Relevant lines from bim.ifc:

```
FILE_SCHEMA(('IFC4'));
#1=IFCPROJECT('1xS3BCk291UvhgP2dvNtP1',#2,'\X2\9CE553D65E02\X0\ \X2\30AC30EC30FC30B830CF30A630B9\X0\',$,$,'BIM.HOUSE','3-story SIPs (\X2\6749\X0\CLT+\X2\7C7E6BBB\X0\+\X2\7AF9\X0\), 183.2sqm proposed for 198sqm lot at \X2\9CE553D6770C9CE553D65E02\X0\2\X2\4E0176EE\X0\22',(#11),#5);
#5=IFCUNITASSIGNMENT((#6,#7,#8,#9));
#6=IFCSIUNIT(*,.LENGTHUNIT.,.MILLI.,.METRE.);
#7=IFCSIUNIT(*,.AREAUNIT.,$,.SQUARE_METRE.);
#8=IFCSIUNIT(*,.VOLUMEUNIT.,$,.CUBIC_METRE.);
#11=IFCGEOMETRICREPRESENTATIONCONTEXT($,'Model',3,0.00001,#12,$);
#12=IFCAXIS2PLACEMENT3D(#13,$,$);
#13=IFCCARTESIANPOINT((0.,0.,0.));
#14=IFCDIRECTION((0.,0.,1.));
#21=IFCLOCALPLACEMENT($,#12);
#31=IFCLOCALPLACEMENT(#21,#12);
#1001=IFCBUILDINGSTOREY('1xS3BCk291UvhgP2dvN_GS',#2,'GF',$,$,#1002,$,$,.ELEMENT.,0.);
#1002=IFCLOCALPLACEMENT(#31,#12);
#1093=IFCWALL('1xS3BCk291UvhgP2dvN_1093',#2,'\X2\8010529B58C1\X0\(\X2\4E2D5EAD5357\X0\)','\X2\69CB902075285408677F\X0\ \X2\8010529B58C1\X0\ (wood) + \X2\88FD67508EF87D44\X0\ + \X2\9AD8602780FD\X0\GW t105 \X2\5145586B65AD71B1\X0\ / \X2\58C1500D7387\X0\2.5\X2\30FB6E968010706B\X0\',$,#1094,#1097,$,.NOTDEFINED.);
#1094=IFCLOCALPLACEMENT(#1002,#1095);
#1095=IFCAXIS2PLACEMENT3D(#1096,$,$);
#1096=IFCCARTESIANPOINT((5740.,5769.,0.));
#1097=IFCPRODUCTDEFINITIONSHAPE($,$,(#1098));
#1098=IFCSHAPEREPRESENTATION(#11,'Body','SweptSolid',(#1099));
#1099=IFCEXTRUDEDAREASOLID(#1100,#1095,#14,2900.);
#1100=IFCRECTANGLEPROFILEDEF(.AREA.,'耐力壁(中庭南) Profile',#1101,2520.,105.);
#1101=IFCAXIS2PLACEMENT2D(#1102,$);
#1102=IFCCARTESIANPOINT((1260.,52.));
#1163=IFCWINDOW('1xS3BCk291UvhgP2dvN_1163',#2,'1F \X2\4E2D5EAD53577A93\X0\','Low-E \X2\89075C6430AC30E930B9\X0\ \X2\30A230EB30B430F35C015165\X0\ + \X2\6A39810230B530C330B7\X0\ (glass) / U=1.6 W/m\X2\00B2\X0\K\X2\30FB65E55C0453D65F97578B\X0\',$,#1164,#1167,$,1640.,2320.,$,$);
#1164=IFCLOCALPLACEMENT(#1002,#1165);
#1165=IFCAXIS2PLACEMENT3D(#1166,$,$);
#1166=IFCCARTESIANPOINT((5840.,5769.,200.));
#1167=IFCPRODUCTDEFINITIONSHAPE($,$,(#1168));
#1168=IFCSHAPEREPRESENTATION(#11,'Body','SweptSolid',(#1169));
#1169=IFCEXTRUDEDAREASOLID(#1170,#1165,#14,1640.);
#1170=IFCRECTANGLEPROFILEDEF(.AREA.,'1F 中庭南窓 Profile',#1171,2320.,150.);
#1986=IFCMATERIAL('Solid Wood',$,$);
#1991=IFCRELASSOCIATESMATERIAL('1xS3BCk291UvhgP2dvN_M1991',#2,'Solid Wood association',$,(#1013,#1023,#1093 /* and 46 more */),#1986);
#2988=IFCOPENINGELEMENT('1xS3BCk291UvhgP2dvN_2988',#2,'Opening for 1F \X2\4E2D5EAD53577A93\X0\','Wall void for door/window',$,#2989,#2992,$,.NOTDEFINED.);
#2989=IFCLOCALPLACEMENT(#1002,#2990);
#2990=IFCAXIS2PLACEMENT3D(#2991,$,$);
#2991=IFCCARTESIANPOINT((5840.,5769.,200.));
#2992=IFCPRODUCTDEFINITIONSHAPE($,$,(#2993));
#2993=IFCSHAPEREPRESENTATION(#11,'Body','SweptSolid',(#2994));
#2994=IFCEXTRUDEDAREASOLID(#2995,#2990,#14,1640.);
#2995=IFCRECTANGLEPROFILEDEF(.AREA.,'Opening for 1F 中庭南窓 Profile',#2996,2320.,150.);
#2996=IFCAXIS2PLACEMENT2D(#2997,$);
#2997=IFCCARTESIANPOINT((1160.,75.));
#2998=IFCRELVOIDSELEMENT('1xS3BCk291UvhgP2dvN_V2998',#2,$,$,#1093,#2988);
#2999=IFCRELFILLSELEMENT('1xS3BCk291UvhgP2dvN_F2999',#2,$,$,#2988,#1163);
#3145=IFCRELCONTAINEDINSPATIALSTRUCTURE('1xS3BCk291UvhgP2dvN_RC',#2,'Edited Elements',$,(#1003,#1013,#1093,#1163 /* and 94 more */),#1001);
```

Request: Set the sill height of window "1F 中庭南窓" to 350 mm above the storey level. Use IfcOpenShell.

```python
import numpy as np
import ifcopenshell
import ifcopenshell.api.geometry
import ifcopenshell.geom
import ifcopenshell.util.element
import ifcopenshell.util.placement
import ifcopenshell.util.shape
import ifcopenshell.util.unit

model = ifcopenshell.open("bim.ifc")
unit_scale = ifcopenshell.util.unit.calculate_unit_scale(model)

window = model.by_id(1163)
opening = window.FillsVoids[0].RelatingOpeningElement
storey = ifcopenshell.util.element.get_container(window, ifc_class="IfcBuildingStorey")
level = ifcopenshell.util.placement.get_local_placement(storey.ObjectPlacement)[2, 3]

# The opening's origin need not be at the sill, so measure its lowest point.
shape = ifcopenshell.geom.create_shape(ifcopenshell.geom.settings(), opening)
bottom = ifcopenshell.util.shape.get_shape_bottom_elevation(shape, shape.geometry) / unit_scale
dz = level + 350.0 - bottom

shift = np.array([0.0, 0.0, dz])
# The window is not placed relative to its opening, so move both.
for product in (opening, window):
    matrix = ifcopenshell.util.placement.get_local_placement(product.ObjectPlacement)
    matrix[:3, 3] += shift
    ifcopenshell.api.geometry.edit_object_placement(model, product=product, matrix=matrix, is_si=False)

print(f"moved by {dz * unit_scale:+.3f} m")

model.write("bim_rev.ifc")
```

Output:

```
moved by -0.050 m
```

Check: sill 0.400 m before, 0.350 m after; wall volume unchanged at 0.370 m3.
